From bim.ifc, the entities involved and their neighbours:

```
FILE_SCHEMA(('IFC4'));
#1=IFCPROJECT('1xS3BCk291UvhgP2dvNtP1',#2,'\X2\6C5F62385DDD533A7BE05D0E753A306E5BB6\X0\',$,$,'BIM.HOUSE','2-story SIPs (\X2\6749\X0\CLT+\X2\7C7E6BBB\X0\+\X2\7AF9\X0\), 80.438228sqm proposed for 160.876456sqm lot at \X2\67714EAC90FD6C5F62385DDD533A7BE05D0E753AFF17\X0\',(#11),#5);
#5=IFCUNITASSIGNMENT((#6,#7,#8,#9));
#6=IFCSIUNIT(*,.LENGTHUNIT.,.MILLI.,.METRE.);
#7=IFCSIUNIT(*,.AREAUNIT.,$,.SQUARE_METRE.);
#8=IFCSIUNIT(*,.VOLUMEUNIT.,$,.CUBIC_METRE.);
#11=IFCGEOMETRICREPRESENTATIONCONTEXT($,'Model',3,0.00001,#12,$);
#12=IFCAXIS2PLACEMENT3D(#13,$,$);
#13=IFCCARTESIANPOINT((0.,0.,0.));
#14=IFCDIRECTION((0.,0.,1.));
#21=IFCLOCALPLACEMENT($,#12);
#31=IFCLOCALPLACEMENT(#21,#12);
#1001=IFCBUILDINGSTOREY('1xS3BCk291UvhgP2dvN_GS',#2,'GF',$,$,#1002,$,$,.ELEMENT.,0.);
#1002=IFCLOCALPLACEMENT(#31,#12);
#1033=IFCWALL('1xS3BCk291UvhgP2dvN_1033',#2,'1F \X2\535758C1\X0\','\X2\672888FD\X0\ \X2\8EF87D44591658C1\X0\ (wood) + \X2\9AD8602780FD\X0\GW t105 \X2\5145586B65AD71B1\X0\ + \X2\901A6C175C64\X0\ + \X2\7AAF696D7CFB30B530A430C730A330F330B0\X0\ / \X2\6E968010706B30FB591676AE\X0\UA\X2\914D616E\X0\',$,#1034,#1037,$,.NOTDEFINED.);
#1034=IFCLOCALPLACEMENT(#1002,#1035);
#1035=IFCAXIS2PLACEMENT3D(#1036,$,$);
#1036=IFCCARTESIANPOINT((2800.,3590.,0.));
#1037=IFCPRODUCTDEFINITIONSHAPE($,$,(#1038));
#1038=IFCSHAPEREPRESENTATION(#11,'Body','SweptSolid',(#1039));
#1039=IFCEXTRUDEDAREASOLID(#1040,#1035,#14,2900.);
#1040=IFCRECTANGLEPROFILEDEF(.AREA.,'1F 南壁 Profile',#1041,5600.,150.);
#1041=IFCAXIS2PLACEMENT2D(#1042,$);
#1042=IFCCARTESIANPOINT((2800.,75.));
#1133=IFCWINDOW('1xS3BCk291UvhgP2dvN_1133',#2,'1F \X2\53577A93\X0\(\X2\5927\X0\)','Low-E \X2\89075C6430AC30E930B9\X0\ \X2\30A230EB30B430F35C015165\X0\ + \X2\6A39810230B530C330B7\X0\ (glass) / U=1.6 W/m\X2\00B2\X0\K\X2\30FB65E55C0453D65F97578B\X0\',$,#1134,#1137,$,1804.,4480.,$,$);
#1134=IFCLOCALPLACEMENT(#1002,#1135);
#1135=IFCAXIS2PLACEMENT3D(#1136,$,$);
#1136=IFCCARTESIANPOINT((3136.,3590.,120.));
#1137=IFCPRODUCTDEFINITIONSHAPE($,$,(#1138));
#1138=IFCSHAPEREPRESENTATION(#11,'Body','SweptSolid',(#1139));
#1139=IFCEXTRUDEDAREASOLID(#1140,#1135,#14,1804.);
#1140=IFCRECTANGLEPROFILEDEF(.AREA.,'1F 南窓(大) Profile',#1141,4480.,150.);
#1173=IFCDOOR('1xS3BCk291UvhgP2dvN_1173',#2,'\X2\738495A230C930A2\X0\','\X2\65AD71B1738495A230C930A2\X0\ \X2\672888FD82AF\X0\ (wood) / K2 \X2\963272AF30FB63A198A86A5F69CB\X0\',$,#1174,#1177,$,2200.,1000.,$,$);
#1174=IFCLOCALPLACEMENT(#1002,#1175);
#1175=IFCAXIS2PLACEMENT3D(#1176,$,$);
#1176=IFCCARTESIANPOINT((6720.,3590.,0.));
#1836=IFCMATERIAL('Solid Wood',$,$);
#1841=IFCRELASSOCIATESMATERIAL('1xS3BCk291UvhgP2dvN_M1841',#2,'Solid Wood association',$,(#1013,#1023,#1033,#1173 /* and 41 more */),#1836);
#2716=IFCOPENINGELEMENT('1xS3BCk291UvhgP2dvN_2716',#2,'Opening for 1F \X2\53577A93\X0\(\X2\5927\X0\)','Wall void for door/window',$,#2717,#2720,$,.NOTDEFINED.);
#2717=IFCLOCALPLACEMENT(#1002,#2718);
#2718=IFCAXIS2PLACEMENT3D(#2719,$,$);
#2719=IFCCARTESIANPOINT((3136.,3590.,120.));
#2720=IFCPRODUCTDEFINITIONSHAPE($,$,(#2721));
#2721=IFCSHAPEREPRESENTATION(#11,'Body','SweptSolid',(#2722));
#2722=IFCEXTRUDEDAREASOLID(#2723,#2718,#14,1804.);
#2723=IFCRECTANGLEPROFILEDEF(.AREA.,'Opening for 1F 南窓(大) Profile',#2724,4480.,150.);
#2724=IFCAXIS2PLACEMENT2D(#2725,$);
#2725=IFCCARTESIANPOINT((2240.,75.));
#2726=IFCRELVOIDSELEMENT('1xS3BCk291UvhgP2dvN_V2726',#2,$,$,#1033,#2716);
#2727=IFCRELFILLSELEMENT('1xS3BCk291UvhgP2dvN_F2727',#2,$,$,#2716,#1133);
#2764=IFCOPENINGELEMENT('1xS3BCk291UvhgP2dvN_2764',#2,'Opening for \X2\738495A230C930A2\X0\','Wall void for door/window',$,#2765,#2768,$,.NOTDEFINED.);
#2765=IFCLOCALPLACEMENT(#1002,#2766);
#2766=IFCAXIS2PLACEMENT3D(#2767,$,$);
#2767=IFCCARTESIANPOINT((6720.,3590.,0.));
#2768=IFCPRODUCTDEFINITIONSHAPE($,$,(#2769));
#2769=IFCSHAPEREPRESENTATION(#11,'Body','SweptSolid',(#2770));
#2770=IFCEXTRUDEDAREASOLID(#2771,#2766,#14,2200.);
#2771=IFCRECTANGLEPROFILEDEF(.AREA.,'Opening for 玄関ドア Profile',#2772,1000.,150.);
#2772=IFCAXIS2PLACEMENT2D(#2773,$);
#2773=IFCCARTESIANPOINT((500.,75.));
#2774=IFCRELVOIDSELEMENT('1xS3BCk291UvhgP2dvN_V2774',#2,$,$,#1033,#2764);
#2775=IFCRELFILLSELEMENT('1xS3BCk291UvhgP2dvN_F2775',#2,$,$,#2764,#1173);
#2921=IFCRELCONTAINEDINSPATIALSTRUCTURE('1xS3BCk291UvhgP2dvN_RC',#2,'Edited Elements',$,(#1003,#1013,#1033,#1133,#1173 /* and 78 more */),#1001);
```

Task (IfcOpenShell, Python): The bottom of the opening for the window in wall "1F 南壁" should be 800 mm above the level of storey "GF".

```python
import numpy as np
import ifcopenshell
import ifcopenshell.api.geometry
import ifcopenshell.geom
import ifcopenshell.util.element
import ifcopenshell.util.placement
import ifcopenshell.util.shape
import ifcopenshell.util.unit

model = ifcopenshell.open("bim.ifc")
unit_scale = ifcopenshell.util.unit.calculate_unit_scale(model)

window = model.by_guid("1xS3BCk291UvhgP2dvN_1133")
opening = window.FillsVoids[0].RelatingOpeningElement
storey = ifcopenshell.util.element.get_container(window, ifc_class="IfcBuildingStorey")
level = ifcopenshell.util.placement.get_local_placement(storey.ObjectPlacement)[2, 3]

# The opening's origin need not be at the sill, so measure its lowest point.
shape = ifcopenshell.geom.create_shape(ifcopenshell.geom.settings(), opening)
bottom = ifcopenshell.util.shape.get_shape_bottom_elevation(shape, shape.geometry) / unit_scale
dz = level + 800.0 - bottom

shift = np.array([0.0, 0.0, dz])
# The window is not placed relative to its opening, so move both.
for product in (opening, window):
    matrix = ifcopenshell.util.placement.get_local_placement(product.ObjectPlacement)
    matrix[:3, 3] += shift
    ifcopenshell.api.geometry.edit_object_placement(model, product=product, matrix=matrix, is_si=False)

print(f"moved by {dz * unit_scale:+.3f} m")

model.write("bim_rev.ifc")
```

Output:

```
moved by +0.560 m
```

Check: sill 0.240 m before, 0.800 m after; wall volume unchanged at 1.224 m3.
